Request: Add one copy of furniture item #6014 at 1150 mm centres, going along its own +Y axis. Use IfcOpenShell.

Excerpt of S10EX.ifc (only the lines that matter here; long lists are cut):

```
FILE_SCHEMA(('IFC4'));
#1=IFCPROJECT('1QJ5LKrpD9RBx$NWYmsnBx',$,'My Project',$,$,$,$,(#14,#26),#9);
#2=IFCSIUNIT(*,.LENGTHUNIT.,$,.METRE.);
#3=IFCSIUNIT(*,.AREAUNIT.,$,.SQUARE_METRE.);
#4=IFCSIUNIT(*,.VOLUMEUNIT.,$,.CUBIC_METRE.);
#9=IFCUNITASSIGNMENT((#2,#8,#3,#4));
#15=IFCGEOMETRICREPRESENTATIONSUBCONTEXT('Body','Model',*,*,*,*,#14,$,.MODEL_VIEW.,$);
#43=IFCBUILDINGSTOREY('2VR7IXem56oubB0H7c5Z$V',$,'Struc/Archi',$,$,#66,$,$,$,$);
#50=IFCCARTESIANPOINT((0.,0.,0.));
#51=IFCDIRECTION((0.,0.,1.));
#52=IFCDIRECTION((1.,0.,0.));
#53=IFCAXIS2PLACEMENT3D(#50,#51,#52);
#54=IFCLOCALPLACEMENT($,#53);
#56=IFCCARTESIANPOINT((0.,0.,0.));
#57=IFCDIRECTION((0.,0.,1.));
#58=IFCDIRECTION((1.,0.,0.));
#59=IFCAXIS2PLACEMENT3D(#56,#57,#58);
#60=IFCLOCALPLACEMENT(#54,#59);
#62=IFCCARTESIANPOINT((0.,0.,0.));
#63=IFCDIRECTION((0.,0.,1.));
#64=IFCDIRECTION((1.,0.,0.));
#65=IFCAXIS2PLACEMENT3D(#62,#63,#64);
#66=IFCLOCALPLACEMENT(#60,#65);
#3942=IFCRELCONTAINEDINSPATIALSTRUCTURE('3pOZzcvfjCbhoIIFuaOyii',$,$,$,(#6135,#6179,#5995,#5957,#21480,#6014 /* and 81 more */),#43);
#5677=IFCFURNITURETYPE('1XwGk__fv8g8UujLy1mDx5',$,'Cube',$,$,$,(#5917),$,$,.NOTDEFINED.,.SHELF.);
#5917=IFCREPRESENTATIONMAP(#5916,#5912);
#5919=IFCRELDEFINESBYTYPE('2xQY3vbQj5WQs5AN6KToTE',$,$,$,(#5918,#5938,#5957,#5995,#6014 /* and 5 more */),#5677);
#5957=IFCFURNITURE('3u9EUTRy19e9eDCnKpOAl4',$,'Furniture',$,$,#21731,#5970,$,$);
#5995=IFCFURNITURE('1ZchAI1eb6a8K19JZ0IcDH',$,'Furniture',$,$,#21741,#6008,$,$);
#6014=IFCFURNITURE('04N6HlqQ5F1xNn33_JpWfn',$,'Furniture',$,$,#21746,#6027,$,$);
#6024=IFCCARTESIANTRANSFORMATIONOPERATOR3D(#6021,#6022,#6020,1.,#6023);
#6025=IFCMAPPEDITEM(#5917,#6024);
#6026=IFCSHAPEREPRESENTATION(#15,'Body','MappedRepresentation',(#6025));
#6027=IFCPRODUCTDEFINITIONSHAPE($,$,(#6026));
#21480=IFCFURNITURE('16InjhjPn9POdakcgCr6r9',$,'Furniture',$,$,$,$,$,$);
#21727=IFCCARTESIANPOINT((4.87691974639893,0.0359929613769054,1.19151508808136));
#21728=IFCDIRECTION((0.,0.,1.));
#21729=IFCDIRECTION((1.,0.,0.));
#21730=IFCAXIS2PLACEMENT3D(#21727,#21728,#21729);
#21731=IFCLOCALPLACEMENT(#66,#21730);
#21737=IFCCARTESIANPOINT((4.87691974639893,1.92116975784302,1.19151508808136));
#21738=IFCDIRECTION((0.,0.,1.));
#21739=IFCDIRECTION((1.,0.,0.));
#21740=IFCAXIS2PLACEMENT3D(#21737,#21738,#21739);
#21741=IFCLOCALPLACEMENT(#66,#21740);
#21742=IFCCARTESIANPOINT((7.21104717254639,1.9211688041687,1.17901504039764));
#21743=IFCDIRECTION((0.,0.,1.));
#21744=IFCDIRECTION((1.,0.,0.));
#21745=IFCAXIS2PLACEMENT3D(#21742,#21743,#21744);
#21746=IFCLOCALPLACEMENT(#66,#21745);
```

```python
import ifcopenshell
import ifcopenshell.api.geometry
import ifcopenshell.api.root
import ifcopenshell.util.element
import ifcopenshell.util.placement

model = ifcopenshell.open("S10EX.ifc")

source = model.by_guid("04N6HlqQ5F1xNn33_JpWfn")
base = ifcopenshell.util.placement.get_local_placement(source.ObjectPlacement)
step = base[:3, 1] * 1.15

for i in range(1, 2):
    copy = ifcopenshell.api.root.copy_class(model, product=source)
    copy.Representation = ifcopenshell.util.element.copy_deep(
        model, source.Representation, exclude=["IfcGeometricRepresentationContext", "IfcRepresentationMap"]
    )
    matrix = base.copy()
    matrix[:3, 3] += i * step
    print("added at", matrix[:3, 3].round(3) + 0.0)
    ifcopenshell.api.geometry.edit_object_placement(model, product=copy, matrix=matrix, is_si=False)

model.write("S10EX_edited.ifc")
```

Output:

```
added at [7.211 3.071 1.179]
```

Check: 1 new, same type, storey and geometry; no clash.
